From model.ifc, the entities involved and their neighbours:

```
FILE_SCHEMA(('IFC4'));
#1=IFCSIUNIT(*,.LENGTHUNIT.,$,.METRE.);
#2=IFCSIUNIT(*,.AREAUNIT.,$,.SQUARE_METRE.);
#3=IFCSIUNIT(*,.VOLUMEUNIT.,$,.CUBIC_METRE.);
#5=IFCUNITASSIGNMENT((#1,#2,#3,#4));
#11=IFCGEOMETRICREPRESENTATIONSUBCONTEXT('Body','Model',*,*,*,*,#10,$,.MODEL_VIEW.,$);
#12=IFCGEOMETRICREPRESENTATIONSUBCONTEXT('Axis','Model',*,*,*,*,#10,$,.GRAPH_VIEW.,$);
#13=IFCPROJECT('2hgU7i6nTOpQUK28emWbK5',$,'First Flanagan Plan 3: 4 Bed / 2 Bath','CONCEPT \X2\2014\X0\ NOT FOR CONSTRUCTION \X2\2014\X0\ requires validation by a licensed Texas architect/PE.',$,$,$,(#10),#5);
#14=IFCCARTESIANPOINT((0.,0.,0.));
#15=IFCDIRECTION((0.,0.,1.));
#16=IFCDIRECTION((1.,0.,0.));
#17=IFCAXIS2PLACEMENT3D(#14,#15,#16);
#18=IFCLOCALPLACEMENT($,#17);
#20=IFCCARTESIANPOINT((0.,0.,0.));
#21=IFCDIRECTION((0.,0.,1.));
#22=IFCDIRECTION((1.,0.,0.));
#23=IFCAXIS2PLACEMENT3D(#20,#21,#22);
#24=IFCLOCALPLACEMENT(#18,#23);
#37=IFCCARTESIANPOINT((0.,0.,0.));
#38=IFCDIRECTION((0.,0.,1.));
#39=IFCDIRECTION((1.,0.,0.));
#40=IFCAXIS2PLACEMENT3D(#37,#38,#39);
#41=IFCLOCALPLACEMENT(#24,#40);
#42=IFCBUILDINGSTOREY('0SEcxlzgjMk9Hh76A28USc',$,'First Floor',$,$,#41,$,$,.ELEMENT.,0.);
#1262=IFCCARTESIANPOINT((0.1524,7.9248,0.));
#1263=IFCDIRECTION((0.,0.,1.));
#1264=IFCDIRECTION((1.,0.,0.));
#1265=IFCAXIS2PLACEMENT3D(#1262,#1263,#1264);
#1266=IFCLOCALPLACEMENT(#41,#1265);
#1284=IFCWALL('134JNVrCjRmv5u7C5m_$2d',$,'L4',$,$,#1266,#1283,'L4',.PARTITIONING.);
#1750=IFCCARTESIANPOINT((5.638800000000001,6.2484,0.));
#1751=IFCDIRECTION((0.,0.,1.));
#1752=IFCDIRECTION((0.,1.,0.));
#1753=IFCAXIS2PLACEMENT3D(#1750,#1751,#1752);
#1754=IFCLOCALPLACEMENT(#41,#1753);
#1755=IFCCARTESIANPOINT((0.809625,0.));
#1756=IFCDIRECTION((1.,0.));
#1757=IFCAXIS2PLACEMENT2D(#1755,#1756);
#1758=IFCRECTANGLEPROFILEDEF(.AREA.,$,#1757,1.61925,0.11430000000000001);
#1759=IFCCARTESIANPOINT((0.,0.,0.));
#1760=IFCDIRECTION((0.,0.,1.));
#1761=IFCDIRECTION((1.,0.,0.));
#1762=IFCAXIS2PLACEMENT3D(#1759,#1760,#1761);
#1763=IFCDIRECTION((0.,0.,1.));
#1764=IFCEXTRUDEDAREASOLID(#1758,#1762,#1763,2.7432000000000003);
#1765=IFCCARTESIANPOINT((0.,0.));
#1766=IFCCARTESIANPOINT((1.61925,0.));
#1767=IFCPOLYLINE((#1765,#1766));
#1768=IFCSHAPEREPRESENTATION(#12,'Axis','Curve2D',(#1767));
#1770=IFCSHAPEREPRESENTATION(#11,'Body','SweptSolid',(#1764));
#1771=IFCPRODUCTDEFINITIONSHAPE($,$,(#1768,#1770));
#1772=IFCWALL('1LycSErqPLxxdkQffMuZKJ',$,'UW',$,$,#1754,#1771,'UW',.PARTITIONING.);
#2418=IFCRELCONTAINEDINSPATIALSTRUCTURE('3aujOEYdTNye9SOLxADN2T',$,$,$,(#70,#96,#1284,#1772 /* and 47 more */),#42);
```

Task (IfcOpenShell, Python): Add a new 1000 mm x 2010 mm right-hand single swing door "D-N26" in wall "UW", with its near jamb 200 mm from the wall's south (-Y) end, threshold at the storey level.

```python
import numpy as np
import ifcopenshell
import ifcopenshell.api.feature
import ifcopenshell.api.geometry
import ifcopenshell.api.root
import ifcopenshell.api.spatial
import ifcopenshell.geom
import ifcopenshell.util.element
import ifcopenshell.util.placement
import ifcopenshell.util.representation
import ifcopenshell.util.shape
import ifcopenshell.util.unit

model = ifcopenshell.open("model.ifc")
unit_scale = ifcopenshell.util.unit.calculate_unit_scale(model)
settings = ifcopenshell.geom.settings()


def volume(element):
    """Net volume in cubic metres, openings subtracted."""
    shape = ifcopenshell.geom.create_shape(settings, element)
    return ifcopenshell.util.shape.get_volume(shape.geometry)


wall = model.by_guid("1LycSErqPLxxdkQffMuZKJ")
storey = ifcopenshell.util.element.get_container(wall, ifc_class="IfcBuildingStorey")
context = ifcopenshell.util.representation.get_context(model, "Model", "Body", "MODEL_VIEW")
before = volume(wall)

width, height, from_end, sill = 1, 2.01, 0.2, 0.0  # metres

# The wall runs along its own X axis, and the end named is its -X end.
wall_shape = ifcopenshell.geom.create_shape(settings, wall)
x, y, z = ifcopenshell.util.shape.get_vertices(wall_shape.geometry).T
start = x.min() + from_end
face, thickness = float(y.min()), float(y.max() - y.min())
wall_matrix = ifcopenshell.util.placement.get_local_placement(wall.ObjectPlacement)
level = ifcopenshell.util.placement.get_local_placement(storey.ObjectPlacement)[2, 3]


def in_wall(x, y):
    """Placement at x, y metres in the wall's axes, at sill height."""
    matrix = wall_matrix.copy()
    matrix[:, 3] = wall_matrix @ np.array([x / unit_scale, y / unit_scale, 0.0, 1.0])
    matrix[2, 3] = level + sill / unit_scale
    return matrix


# Opening: a box that overshoots both wall faces by 50 mm.
opening = ifcopenshell.api.root.create_entity(model, ifc_class="IfcOpeningElement", predefined_type="OPENING")
box = ifcopenshell.api.geometry.add_wall_representation(
    model, context=context, length=width, height=height, thickness=thickness + 0.1
)
ifcopenshell.api.geometry.assign_representation(model, product=opening, representation=box)
ifcopenshell.api.geometry.edit_object_placement(model, product=opening, matrix=in_wall(start, face - 0.05), is_si=False)
ifcopenshell.api.feature.add_feature(model, feature=opening, element=wall)

door = ifcopenshell.api.root.create_entity(model, ifc_class="IfcDoor", name="D-N26", predefined_type="DOOR")
door.OverallWidth, door.OverallHeight = width / unit_scale, height / unit_scale
door.OperationType = "SINGLE_SWING_RIGHT"
body = ifcopenshell.api.geometry.add_door_representation(
    model,
    context=context,
    overall_width=door.OverallWidth,
    overall_height=door.OverallHeight,
    operation_type="SINGLE_SWING_RIGHT",
    lining_properties={"LiningDepth": thickness / unit_scale, "ThresholdDepth": thickness / unit_scale},
)
ifcopenshell.api.geometry.assign_representation(model, product=door, representation=body)
ifcopenshell.api.spatial.assign_container(model, products=[door], relating_structure=storey)
ifcopenshell.api.feature.add_filling(model, opening=opening, element=door)

# The lining spans the wall, so the door starts at the wall face.
ifcopenshell.api.geometry.edit_object_placement(model, product=door, matrix=in_wall(start, face), is_si=False)

after = volume(wall)

print(f"wall volume {before:.3f} -> {after:.3f} m3")

model.write("model_rev.ifc")
```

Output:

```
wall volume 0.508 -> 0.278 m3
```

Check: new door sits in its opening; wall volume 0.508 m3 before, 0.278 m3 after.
